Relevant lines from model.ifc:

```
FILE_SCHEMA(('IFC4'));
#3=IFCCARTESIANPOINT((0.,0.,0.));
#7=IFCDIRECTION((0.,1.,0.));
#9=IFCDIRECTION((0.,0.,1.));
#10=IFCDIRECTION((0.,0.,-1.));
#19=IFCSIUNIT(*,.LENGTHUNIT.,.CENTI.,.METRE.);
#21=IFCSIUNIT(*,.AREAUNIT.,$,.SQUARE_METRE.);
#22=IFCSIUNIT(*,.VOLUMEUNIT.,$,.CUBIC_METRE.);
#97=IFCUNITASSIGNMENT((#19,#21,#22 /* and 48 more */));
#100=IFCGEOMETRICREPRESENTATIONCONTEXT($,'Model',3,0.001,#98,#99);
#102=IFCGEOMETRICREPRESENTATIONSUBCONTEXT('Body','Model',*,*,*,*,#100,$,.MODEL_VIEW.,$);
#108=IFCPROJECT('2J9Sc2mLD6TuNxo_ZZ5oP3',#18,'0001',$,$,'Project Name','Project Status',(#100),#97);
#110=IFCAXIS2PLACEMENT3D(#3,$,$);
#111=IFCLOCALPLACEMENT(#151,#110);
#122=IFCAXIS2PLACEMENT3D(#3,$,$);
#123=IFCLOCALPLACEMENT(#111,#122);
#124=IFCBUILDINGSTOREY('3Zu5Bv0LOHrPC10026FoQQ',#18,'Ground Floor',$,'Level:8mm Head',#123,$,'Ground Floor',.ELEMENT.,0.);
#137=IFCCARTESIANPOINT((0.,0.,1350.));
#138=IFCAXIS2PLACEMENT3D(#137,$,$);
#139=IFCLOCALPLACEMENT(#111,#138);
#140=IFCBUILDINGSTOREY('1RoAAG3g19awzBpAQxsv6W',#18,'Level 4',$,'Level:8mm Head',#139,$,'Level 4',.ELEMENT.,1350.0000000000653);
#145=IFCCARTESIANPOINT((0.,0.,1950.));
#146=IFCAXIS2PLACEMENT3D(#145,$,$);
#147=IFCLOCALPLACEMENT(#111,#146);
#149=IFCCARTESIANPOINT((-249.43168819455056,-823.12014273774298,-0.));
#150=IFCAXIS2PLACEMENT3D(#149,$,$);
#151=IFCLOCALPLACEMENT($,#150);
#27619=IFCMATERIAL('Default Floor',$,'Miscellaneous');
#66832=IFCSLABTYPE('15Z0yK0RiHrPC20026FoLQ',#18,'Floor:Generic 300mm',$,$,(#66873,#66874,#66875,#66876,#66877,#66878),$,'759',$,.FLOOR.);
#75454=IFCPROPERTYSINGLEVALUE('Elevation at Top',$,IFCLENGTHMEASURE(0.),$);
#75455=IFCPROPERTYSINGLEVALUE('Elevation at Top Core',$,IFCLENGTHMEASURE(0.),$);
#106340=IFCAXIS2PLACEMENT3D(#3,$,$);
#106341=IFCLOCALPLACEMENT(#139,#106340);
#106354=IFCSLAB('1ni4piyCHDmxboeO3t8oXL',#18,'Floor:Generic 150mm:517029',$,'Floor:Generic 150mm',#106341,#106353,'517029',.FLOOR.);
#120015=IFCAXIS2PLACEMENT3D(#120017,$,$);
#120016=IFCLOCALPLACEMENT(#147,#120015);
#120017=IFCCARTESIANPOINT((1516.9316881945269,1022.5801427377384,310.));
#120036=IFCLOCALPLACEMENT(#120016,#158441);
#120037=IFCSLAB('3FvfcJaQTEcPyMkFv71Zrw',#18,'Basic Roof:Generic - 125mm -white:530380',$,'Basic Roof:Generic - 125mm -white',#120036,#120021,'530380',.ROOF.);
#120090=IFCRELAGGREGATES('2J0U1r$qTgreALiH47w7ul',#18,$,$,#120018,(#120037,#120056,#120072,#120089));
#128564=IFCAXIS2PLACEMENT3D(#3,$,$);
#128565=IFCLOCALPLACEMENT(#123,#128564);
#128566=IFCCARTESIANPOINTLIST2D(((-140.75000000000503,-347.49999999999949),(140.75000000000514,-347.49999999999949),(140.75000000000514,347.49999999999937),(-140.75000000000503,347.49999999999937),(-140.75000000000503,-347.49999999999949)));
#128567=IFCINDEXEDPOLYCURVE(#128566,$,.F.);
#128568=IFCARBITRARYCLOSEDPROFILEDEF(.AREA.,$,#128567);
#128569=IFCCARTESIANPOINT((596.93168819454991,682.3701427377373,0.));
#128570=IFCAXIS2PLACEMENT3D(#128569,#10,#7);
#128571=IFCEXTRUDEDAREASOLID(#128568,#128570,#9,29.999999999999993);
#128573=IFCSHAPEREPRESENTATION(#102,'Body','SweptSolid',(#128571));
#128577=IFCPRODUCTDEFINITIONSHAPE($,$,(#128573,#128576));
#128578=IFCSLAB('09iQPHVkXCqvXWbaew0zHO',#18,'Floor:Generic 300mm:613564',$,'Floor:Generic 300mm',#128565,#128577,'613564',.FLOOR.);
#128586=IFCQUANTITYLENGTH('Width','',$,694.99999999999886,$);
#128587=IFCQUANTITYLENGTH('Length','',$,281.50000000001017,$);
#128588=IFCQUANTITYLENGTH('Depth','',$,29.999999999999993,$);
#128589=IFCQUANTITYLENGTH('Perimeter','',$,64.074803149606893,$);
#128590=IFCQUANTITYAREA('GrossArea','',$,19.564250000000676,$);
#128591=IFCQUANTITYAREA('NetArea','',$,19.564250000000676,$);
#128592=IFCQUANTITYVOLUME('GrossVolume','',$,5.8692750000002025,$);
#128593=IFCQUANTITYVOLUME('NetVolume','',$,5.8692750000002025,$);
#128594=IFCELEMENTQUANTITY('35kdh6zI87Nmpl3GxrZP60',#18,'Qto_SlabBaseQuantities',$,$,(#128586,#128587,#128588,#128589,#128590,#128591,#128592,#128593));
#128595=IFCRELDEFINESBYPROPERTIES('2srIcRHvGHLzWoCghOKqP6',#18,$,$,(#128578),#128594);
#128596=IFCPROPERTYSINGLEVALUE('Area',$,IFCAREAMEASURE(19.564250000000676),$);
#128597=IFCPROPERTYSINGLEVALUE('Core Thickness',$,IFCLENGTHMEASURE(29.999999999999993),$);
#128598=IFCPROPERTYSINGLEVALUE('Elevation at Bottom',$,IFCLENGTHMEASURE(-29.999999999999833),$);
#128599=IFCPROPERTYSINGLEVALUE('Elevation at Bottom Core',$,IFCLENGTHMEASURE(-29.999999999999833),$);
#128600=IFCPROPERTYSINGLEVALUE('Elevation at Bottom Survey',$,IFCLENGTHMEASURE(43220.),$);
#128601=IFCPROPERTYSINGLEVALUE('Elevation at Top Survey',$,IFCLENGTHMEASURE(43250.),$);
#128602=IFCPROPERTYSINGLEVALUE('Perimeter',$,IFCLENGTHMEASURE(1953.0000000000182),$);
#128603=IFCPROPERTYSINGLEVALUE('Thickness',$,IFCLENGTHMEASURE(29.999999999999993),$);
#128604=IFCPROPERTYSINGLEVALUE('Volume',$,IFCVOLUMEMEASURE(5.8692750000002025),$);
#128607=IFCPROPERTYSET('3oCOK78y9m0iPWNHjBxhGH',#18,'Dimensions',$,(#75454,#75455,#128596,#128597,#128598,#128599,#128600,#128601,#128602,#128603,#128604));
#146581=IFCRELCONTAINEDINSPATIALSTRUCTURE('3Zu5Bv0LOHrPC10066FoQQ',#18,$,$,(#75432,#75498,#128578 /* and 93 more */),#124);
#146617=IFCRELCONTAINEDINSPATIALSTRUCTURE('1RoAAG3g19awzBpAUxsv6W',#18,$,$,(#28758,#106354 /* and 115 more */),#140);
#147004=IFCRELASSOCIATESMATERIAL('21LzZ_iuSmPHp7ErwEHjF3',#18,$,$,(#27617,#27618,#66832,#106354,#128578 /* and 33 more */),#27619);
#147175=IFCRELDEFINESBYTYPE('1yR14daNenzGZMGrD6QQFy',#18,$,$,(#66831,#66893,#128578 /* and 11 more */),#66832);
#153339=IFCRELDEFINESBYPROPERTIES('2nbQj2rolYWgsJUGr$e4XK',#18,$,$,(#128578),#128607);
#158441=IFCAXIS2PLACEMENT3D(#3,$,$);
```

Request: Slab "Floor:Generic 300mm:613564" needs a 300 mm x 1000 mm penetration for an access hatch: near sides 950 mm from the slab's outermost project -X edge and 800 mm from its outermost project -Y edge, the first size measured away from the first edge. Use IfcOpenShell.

```python
import numpy as np
import ifcopenshell
import ifcopenshell.api.feature
import ifcopenshell.api.geometry
import ifcopenshell.api.pset
import ifcopenshell.api.root
import ifcopenshell.geom
import ifcopenshell.util.element
import ifcopenshell.util.placement
import ifcopenshell.util.representation
import ifcopenshell.util.shape
import ifcopenshell.util.unit

model = ifcopenshell.open("model.ifc")
unit_scale = ifcopenshell.util.unit.calculate_unit_scale(model)
area_scale = ifcopenshell.util.unit.calculate_unit_scale(model, "AREAUNIT")
volume_scale = ifcopenshell.util.unit.calculate_unit_scale(model, "VOLUMEUNIT")
settings = ifcopenshell.geom.settings()


def volume(element):
    """Net volume in cubic metres, openings subtracted."""
    shape = ifcopenshell.geom.create_shape(settings, element)
    return ifcopenshell.util.shape.get_volume(shape.geometry)


slab = model.by_guid("09iQPHVkXCqvXWbaew0zHO")
before = volume(slab)

# Extent in the slab's own axes, in metres. The edges named are its -X and -Y sides.
slab_shape = ifcopenshell.geom.create_shape(settings, slab)
vertices = ifcopenshell.util.shape.get_vertices(slab_shape.geometry)
x_min, y_min, bottom = vertices.min(axis=0)
top = vertices[:, 2].max()

opening = ifcopenshell.api.root.create_entity(model, ifc_class="IfcOpeningElement", name="Access hatch opening", predefined_type="OPENING")
context = ifcopenshell.util.representation.get_context(model, "Model", "Body", "MODEL_VIEW")
width, depth = 0.3, 1
outline = [(0.0, 0.0), (width, 0.0), (width, depth), (0.0, depth), (0.0, 0.0)]
# Overshoot both faces by 50 mm so the cut is clean.
shape = ifcopenshell.api.geometry.add_slab_representation(
    model, context=context, depth=top - bottom + 0.1, polyline=outline
)
ifcopenshell.api.geometry.assign_representation(model, product=opening, representation=shape)

matrix = ifcopenshell.util.placement.get_local_placement(slab.ObjectPlacement)
matrix[:, 3] = matrix @ np.append(np.array([x_min + 0.95, y_min + 0.8, bottom - 0.05]) / unit_scale, 1.0)
ifcopenshell.api.geometry.edit_object_placement(model, product=opening, matrix=matrix, is_si=False)
ifcopenshell.api.feature.add_feature(model, feature=opening, element=slab)

after = volume(slab)

# Update the slab's stored quantities.
qto = model.by_id(ifcopenshell.util.element.get_pset(slab, "Qto_SlabBaseQuantities", should_inherit=False)["id"])
ifcopenshell.api.pset.edit_qto(model, qto=qto, properties={
    "NetArea": after / (top - bottom) / area_scale,
    "NetVolume": after / volume_scale,
})
pset = model.by_id(ifcopenshell.util.element.get_pset(slab, "Dimensions", should_inherit=False)["id"])
ifcopenshell.api.pset.edit_pset(model, pset=pset, properties={
    "Area": model.create_entity("IfcAreaMeasure", after / (top - bottom) / area_scale),
    "Volume": model.create_entity("IfcVolumeMeasure", after / volume_scale),
})

print(f"slab volume {before:.3f} -> {after:.3f} m3")

model.write("model-out.ifc")
```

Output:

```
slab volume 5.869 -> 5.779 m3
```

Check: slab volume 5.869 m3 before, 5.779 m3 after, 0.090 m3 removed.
